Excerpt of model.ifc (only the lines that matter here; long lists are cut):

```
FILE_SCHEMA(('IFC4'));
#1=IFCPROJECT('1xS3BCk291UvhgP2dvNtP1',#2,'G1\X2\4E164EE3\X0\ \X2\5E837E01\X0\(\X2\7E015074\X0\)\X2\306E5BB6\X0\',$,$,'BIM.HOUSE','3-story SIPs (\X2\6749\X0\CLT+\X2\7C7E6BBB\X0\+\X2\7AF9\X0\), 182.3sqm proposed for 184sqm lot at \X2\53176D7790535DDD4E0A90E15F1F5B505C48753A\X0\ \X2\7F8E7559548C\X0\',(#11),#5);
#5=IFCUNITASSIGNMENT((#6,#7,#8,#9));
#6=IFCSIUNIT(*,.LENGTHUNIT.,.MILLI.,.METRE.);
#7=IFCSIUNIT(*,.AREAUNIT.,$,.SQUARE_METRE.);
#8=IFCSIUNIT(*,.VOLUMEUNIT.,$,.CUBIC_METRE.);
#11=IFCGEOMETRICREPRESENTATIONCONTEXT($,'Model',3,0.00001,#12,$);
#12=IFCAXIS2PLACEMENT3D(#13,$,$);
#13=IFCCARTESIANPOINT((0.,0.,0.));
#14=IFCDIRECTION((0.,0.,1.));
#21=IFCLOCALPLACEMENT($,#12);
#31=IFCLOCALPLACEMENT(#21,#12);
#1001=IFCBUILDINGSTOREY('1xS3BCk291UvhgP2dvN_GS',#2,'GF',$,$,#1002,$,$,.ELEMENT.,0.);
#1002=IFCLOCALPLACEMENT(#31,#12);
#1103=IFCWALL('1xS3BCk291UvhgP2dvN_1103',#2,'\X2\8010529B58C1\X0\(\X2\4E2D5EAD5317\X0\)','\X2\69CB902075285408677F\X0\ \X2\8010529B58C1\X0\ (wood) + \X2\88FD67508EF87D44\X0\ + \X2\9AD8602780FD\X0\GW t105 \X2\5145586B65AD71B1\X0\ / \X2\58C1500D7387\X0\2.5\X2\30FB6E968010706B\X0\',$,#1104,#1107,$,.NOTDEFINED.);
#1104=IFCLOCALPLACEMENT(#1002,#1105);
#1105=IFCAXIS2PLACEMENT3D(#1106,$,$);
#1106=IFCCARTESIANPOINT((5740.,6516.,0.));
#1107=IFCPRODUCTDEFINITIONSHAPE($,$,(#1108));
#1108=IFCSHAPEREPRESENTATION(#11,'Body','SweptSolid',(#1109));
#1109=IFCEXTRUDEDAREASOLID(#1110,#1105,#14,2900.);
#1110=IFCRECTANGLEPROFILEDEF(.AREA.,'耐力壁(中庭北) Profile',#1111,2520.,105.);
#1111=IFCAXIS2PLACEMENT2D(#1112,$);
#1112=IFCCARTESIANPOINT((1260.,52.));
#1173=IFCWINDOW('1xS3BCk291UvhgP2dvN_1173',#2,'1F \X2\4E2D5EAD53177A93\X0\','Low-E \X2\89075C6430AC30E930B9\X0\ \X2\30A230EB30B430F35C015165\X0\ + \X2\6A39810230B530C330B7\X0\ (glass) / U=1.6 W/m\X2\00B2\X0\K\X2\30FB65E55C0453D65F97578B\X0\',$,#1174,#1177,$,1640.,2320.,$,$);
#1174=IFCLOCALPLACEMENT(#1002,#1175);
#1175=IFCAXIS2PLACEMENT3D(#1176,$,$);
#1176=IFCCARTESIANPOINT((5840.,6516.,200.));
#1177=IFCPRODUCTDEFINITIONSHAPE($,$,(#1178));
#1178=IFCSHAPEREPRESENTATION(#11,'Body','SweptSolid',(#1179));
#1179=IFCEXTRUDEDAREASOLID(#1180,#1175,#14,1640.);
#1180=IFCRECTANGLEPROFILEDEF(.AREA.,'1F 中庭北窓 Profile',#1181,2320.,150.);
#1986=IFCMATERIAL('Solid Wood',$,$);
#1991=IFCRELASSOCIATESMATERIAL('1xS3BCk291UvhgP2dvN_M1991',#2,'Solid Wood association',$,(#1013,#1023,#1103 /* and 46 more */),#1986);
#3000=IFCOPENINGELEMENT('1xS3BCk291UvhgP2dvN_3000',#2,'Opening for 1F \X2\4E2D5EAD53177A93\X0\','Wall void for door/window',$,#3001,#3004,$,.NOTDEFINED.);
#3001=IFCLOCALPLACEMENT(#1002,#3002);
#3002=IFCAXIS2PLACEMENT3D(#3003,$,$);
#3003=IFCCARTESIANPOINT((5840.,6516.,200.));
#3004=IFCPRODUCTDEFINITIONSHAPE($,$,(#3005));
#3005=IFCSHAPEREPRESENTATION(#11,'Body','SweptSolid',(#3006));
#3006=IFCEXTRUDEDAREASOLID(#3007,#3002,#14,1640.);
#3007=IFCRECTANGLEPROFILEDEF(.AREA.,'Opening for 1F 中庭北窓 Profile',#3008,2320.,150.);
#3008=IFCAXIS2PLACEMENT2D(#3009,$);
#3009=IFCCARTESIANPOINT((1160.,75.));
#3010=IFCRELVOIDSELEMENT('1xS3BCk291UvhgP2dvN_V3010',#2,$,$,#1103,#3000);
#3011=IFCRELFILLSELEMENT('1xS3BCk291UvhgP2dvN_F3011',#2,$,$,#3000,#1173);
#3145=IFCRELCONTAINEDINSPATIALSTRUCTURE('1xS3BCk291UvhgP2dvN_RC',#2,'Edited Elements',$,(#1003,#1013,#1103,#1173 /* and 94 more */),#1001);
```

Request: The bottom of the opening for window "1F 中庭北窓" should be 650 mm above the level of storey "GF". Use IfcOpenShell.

```python
import numpy as np
import ifcopenshell
import ifcopenshell.api.geometry
import ifcopenshell.geom
import ifcopenshell.util.element
import ifcopenshell.util.placement
import ifcopenshell.util.shape
import ifcopenshell.util.unit

model = ifcopenshell.open("model.ifc")
unit_scale = ifcopenshell.util.unit.calculate_unit_scale(model)

window = model.by_guid("1xS3BCk291UvhgP2dvN_1173")
opening = window.FillsVoids[0].RelatingOpeningElement
storey = ifcopenshell.util.element.get_container(window, ifc_class="IfcBuildingStorey")
level = ifcopenshell.util.placement.get_local_placement(storey.ObjectPlacement)[2, 3]

# The opening's origin need not be at the sill, so measure its lowest point.
shape = ifcopenshell.geom.create_shape(ifcopenshell.geom.settings(), opening)
bottom = ifcopenshell.util.shape.get_shape_bottom_elevation(shape, shape.geometry) / unit_scale
dz = level + 650.0 - bottom

shift = np.array([0.0, 0.0, dz])
# The window is not placed relative to its opening, so move both.
for product in (opening, window):
    matrix = ifcopenshell.util.placement.get_local_placement(product.ObjectPlacement)
    matrix[:3, 3] += shift
    ifcopenshell.api.geometry.edit_object_placement(model, product=product, matrix=matrix, is_si=False)

print(f"moved by {dz * unit_scale:+.3f} m")

model.write("model-out.ifc")
```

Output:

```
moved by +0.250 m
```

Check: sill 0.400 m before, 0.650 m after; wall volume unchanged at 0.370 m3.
